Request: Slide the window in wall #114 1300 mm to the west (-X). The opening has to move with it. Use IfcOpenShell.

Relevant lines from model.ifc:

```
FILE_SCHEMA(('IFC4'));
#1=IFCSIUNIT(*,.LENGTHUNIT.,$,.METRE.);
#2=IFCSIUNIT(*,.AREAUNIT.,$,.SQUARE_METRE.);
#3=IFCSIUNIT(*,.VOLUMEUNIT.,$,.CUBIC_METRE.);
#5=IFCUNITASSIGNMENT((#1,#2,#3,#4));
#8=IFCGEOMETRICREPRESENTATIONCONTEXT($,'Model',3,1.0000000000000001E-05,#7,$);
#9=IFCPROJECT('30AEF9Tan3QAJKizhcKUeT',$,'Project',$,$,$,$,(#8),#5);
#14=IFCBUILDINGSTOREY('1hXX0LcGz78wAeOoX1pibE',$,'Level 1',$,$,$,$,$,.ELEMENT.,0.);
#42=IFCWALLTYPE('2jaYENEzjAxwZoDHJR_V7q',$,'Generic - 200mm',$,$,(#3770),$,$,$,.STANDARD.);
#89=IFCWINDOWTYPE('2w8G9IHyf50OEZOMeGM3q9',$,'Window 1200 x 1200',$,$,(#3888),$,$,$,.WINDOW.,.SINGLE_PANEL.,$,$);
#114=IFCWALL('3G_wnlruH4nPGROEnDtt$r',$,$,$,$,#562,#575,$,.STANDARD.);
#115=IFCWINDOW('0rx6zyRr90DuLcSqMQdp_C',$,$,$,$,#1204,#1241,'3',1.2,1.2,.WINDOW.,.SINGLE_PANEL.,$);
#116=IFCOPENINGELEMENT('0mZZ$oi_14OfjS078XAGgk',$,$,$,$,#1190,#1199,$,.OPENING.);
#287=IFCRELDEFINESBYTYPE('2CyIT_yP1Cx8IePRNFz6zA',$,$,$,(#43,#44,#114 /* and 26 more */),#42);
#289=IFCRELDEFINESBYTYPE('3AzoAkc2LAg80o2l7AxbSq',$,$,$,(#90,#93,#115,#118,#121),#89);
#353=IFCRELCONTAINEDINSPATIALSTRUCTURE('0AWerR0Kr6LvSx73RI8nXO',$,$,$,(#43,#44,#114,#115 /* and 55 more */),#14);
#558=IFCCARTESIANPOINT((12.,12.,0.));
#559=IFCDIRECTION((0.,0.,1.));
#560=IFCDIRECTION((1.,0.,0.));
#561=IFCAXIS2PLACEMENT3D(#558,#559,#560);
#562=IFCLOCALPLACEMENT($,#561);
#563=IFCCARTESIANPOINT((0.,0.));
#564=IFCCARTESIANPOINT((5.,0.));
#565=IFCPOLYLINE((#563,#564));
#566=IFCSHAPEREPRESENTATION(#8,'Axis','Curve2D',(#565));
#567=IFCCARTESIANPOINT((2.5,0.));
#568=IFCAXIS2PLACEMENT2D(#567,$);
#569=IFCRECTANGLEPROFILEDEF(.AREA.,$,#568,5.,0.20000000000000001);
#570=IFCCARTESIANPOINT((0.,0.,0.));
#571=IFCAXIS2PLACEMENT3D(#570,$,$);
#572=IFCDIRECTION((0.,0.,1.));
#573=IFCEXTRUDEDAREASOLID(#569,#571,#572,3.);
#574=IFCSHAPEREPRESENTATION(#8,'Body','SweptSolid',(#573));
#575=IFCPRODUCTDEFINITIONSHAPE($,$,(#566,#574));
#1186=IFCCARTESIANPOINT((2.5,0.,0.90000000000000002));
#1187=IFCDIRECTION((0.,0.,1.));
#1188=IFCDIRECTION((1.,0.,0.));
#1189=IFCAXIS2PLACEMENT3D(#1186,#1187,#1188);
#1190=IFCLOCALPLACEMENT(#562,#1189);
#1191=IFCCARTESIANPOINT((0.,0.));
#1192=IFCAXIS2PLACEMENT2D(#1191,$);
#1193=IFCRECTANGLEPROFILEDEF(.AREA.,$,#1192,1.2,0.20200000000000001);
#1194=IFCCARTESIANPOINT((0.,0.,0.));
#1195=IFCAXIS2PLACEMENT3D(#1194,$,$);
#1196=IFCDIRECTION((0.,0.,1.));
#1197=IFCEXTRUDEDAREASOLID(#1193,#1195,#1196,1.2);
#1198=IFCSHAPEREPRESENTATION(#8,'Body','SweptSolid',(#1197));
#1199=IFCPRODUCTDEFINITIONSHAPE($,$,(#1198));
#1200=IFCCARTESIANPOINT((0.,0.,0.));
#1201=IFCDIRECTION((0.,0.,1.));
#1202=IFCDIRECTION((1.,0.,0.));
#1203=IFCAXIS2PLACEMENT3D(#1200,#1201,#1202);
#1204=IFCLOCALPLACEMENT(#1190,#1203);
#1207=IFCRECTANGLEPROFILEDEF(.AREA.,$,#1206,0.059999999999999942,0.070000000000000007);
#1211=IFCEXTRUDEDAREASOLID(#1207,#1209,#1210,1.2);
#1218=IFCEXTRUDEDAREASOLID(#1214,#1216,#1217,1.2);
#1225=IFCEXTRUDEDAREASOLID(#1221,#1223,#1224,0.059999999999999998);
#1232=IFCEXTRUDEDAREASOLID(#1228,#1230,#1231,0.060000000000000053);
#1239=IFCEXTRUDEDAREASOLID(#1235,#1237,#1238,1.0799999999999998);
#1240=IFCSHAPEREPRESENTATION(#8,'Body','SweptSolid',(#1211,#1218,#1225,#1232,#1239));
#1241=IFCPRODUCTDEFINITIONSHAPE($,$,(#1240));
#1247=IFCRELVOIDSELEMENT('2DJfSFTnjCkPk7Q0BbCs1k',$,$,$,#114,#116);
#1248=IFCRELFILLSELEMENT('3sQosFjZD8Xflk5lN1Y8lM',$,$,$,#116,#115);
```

```python
import ifcopenshell
import ifcopenshell.api.geometry
import ifcopenshell.util.placement

model = ifcopenshell.open("model.ifc")

window = model.by_guid("0rx6zyRr90DuLcSqMQdp_C")
opening = window.FillsVoids[0].RelatingOpeningElement
wall = opening.VoidsElements[0].RelatingBuildingElement

wall_matrix = ifcopenshell.util.placement.get_local_placement(wall.ObjectPlacement)
shift = wall_matrix[:3, 0] * -1.3
before = ifcopenshell.util.placement.get_local_placement(window.ObjectPlacement)[:3, 3].copy()

# The window is placed relative to its opening, so it follows when the opening moves.
matrix = ifcopenshell.util.placement.get_local_placement(opening.ObjectPlacement)
matrix[:3, 3] += shift
ifcopenshell.api.geometry.edit_object_placement(
    model, product=opening, matrix=matrix, is_si=False, should_transform_children=True
)

after = ifcopenshell.util.placement.get_local_placement(window.ObjectPlacement)[:3, 3]
print("window moved by", (after - before).round(3) + 0.0)

model.write("model_updated.ifc")
```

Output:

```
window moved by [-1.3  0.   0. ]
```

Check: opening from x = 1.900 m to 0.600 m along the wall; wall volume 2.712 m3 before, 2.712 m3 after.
